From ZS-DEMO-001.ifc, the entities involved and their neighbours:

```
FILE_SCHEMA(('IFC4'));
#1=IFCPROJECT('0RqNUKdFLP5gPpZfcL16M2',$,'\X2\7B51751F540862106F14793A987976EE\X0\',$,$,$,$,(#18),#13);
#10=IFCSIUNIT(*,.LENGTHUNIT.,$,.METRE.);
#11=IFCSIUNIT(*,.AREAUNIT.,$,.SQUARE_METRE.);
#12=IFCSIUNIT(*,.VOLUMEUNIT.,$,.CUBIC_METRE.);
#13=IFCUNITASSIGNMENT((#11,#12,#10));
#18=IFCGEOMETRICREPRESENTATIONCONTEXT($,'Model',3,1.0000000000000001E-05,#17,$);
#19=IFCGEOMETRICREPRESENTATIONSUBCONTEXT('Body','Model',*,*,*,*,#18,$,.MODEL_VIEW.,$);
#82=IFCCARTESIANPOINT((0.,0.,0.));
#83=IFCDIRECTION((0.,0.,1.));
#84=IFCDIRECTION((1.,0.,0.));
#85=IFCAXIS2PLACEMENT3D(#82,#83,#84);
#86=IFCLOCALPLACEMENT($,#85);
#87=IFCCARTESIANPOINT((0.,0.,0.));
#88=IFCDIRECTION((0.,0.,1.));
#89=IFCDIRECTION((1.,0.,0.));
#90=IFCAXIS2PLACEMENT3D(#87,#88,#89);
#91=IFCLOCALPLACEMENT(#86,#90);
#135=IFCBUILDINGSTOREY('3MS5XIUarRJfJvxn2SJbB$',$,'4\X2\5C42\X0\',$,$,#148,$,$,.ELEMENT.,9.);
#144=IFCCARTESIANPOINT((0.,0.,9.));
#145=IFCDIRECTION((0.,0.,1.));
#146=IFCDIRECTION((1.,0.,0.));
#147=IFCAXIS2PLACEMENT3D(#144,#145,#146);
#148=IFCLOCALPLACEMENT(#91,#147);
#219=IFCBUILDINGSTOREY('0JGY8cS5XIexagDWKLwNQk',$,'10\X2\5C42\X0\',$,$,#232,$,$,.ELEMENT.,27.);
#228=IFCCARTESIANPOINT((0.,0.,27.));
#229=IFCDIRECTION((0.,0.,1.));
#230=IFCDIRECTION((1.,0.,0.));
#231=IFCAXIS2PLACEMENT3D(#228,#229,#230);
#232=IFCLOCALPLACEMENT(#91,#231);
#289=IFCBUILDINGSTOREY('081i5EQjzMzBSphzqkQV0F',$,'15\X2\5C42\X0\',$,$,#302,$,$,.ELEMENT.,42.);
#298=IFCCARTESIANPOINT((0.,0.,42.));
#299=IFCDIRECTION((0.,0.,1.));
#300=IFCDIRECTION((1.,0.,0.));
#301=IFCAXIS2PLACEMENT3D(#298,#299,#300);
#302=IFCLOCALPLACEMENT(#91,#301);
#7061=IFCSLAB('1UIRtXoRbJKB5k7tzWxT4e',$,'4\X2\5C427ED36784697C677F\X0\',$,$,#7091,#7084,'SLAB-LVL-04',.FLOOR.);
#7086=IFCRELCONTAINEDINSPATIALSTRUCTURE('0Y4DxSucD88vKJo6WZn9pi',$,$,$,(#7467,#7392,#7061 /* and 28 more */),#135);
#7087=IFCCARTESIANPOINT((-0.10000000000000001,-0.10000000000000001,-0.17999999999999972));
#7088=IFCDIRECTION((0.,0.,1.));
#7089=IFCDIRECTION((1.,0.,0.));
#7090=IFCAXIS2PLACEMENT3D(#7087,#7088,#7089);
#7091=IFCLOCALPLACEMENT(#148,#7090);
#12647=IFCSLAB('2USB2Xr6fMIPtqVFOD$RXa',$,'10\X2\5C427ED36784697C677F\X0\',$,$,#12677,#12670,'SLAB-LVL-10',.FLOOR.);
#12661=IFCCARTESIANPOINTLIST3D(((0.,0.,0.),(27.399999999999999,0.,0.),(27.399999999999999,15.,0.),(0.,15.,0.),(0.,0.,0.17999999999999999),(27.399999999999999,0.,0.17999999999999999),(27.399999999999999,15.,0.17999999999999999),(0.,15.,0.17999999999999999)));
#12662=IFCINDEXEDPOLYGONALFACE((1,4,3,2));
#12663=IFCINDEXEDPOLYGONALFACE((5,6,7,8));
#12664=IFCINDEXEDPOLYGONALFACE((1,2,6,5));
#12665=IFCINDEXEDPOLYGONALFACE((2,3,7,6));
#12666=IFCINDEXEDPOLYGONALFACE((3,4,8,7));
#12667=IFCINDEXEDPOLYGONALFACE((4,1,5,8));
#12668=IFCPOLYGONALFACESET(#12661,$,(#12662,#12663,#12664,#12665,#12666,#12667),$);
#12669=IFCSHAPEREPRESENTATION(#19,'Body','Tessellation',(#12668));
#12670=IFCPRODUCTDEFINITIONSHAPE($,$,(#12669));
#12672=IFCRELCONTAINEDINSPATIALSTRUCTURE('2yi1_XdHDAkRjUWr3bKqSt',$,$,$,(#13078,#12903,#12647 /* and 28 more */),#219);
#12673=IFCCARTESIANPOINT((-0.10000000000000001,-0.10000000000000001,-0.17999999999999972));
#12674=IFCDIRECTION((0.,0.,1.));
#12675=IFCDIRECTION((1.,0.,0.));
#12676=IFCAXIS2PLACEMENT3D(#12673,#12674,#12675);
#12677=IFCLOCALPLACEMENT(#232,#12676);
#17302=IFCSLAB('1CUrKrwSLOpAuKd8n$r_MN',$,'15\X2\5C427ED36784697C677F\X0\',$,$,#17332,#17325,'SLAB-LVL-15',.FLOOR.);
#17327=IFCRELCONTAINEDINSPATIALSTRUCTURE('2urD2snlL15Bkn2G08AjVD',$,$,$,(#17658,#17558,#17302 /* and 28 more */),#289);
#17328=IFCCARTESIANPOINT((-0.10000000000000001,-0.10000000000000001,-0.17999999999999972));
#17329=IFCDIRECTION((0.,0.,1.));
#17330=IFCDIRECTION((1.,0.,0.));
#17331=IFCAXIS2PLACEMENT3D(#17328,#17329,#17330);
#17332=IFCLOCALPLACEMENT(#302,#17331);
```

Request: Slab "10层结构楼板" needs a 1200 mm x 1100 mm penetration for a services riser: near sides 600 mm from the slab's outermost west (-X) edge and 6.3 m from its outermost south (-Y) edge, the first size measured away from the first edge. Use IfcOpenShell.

```python
import numpy as np
import ifcopenshell
import ifcopenshell.api.feature
import ifcopenshell.api.geometry
import ifcopenshell.api.root
import ifcopenshell.geom
import ifcopenshell.util.placement
import ifcopenshell.util.representation
import ifcopenshell.util.shape
import ifcopenshell.util.unit

model = ifcopenshell.open("ZS-DEMO-001.ifc")
unit_scale = ifcopenshell.util.unit.calculate_unit_scale(model)
settings = ifcopenshell.geom.settings()


def volume(element):
    """Net volume in cubic metres, openings subtracted."""
    shape = ifcopenshell.geom.create_shape(settings, element)
    return ifcopenshell.util.shape.get_volume(shape.geometry)


slab = model.by_guid("2USB2Xr6fMIPtqVFOD$RXa")
before = volume(slab)

# Extent in the slab's own axes, in metres. The edges named are its -X and -Y sides.
slab_shape = ifcopenshell.geom.create_shape(settings, slab)
vertices = ifcopenshell.util.shape.get_vertices(slab_shape.geometry)
x_min, y_min, bottom = vertices.min(axis=0)
top = vertices[:, 2].max()

opening = ifcopenshell.api.root.create_entity(model, ifc_class="IfcOpeningElement", name="Services riser opening", predefined_type="OPENING")
context = ifcopenshell.util.representation.get_context(model, "Model", "Body", "MODEL_VIEW")
width, depth = 1.2, 1.1
outline = [(0.0, 0.0), (width, 0.0), (width, depth), (0.0, depth), (0.0, 0.0)]
# Overshoot both faces by 50 mm so the cut is clean.
shape = ifcopenshell.api.geometry.add_slab_representation(
    model, context=context, depth=top - bottom + 0.1, polyline=outline
)
ifcopenshell.api.geometry.assign_representation(model, product=opening, representation=shape)

matrix = ifcopenshell.util.placement.get_local_placement(slab.ObjectPlacement)
matrix[:, 3] = matrix @ np.append(np.array([x_min + 0.6, y_min + 6.3, bottom - 0.05]) / unit_scale, 1.0)
ifcopenshell.api.geometry.edit_object_placement(model, product=opening, matrix=matrix, is_si=False)
ifcopenshell.api.feature.add_feature(model, feature=opening, element=slab)

after = volume(slab)

print(f"slab volume {before:.3f} -> {after:.3f} m3")

model.write("ZS-DEMO-001_rev.ifc")
```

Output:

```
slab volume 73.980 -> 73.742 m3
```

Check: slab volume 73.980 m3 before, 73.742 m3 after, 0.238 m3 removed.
